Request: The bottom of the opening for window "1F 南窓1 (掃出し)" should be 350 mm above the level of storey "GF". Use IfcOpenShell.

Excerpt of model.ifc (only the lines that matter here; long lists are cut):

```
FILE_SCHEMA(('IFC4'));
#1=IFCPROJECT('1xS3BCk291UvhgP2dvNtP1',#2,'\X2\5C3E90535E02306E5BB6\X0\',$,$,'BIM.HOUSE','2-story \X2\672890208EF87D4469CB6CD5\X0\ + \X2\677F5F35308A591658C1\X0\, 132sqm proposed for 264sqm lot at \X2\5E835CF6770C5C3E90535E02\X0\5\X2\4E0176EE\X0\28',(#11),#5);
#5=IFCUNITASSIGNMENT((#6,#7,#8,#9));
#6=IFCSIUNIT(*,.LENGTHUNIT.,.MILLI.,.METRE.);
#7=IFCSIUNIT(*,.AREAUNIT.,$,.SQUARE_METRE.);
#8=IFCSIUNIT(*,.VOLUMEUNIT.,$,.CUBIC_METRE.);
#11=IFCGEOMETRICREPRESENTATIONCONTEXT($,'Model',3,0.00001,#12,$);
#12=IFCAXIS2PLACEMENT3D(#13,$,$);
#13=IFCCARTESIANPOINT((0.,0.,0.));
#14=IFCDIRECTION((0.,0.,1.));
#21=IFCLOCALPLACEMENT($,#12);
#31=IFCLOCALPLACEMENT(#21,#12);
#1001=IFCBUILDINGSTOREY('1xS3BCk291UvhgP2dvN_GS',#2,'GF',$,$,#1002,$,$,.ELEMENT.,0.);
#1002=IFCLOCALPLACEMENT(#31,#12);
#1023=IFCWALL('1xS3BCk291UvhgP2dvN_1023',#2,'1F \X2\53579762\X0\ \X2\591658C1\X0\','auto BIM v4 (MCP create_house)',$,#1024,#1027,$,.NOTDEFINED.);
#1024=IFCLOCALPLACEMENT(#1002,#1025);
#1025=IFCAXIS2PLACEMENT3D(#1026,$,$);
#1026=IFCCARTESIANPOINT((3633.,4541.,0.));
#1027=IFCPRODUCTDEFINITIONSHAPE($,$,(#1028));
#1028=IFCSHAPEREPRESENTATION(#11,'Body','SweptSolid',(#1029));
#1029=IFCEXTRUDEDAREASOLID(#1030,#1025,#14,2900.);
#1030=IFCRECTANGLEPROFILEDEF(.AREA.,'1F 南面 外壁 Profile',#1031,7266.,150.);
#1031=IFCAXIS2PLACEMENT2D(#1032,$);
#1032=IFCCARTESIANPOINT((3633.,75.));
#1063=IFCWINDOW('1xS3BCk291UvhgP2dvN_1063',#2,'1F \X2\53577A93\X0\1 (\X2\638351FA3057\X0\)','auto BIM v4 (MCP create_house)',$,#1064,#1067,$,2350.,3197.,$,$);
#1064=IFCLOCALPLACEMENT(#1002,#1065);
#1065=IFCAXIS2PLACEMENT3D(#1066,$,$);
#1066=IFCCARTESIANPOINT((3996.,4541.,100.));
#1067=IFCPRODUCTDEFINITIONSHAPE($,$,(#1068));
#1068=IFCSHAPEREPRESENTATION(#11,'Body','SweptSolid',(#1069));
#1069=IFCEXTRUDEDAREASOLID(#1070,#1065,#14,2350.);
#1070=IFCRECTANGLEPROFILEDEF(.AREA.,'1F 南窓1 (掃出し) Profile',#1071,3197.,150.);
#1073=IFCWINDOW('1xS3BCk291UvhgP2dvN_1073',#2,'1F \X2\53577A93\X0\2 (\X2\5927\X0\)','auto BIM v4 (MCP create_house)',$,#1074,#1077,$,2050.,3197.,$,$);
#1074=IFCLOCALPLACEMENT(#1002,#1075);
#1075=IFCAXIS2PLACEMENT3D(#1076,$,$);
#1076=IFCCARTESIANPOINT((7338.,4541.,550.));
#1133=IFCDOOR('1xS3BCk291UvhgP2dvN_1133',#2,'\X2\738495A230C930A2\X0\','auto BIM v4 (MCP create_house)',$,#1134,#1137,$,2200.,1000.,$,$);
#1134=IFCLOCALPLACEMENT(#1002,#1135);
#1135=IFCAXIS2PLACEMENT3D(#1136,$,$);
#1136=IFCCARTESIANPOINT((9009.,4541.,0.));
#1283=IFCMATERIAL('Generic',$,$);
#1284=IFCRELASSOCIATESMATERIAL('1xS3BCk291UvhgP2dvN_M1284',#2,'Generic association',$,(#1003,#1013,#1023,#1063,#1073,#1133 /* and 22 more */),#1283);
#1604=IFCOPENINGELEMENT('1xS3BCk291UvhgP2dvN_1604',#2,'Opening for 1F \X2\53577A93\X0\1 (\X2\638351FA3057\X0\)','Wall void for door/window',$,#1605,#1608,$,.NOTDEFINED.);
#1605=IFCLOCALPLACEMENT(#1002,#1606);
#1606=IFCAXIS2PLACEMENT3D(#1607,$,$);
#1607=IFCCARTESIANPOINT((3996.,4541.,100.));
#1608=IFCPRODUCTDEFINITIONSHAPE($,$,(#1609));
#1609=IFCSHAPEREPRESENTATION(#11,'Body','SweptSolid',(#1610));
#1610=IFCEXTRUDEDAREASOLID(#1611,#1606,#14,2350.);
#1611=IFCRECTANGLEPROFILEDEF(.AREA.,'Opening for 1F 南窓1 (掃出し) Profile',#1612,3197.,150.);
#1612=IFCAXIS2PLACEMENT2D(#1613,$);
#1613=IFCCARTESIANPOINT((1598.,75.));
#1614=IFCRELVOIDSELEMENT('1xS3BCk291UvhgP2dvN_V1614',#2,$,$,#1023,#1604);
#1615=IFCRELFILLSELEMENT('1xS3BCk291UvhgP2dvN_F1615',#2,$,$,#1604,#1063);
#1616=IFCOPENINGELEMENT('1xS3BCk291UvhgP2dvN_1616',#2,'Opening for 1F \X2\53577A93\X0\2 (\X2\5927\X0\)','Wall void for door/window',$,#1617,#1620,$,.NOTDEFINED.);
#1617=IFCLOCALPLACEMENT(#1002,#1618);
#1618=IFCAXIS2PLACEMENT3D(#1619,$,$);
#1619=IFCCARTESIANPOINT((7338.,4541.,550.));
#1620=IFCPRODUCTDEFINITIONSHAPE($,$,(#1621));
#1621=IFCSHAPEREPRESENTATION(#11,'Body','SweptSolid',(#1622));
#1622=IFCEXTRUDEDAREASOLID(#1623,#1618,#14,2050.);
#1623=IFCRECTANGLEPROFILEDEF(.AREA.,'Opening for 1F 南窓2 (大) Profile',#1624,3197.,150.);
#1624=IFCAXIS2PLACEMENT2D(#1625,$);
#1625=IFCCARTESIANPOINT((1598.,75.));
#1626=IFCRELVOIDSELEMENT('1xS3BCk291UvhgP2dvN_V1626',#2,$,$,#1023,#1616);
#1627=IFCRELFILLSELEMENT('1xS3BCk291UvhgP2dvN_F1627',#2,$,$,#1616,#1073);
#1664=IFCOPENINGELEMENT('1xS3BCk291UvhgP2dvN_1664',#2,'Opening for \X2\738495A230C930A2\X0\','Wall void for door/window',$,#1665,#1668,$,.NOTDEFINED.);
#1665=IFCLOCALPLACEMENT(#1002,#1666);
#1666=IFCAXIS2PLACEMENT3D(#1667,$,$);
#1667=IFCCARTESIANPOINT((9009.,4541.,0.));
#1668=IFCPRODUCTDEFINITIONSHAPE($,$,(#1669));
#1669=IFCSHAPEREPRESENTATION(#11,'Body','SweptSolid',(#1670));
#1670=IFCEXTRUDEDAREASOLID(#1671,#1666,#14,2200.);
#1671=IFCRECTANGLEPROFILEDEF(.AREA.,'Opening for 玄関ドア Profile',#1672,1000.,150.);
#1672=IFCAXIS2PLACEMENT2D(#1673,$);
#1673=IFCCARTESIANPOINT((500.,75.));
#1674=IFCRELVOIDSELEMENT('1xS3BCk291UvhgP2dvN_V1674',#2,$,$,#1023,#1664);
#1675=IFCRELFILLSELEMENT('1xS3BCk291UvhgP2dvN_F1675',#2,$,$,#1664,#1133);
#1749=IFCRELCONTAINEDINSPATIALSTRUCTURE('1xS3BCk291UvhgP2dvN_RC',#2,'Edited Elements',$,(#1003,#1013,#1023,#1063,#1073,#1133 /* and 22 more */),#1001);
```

```python
import numpy as np
import ifcopenshell
import ifcopenshell.api.geometry
import ifcopenshell.geom
import ifcopenshell.util.element
import ifcopenshell.util.placement
import ifcopenshell.util.shape
import ifcopenshell.util.unit

model = ifcopenshell.open("model.ifc")
unit_scale = ifcopenshell.util.unit.calculate_unit_scale(model)

window = model.by_id(1063)
opening = window.FillsVoids[0].RelatingOpeningElement
storey = ifcopenshell.util.element.get_container(window, ifc_class="IfcBuildingStorey")
level = ifcopenshell.util.placement.get_local_placement(storey.ObjectPlacement)[2, 3]

# The opening's origin need not be at the sill, so measure its lowest point.
shape = ifcopenshell.geom.create_shape(ifcopenshell.geom.settings(), opening)
bottom = ifcopenshell.util.shape.get_shape_bottom_elevation(shape, shape.geometry) / unit_scale
dz = level + 0.35 / unit_scale - bottom

shift = np.array([0.0, 0.0, dz])
# The window is not placed relative to its opening, so move both.
for product in (opening, window):
    matrix = ifcopenshell.util.placement.get_local_placement(product.ObjectPlacement)
    matrix[:3, 3] += shift
    ifcopenshell.api.geometry.edit_object_placement(model, product=product, matrix=matrix, is_si=False)

print(f"moved by {dz * unit_scale:+.3f} m")

model.write("model_rev.ifc")
```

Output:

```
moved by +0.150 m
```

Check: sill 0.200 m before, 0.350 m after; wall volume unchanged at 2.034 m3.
